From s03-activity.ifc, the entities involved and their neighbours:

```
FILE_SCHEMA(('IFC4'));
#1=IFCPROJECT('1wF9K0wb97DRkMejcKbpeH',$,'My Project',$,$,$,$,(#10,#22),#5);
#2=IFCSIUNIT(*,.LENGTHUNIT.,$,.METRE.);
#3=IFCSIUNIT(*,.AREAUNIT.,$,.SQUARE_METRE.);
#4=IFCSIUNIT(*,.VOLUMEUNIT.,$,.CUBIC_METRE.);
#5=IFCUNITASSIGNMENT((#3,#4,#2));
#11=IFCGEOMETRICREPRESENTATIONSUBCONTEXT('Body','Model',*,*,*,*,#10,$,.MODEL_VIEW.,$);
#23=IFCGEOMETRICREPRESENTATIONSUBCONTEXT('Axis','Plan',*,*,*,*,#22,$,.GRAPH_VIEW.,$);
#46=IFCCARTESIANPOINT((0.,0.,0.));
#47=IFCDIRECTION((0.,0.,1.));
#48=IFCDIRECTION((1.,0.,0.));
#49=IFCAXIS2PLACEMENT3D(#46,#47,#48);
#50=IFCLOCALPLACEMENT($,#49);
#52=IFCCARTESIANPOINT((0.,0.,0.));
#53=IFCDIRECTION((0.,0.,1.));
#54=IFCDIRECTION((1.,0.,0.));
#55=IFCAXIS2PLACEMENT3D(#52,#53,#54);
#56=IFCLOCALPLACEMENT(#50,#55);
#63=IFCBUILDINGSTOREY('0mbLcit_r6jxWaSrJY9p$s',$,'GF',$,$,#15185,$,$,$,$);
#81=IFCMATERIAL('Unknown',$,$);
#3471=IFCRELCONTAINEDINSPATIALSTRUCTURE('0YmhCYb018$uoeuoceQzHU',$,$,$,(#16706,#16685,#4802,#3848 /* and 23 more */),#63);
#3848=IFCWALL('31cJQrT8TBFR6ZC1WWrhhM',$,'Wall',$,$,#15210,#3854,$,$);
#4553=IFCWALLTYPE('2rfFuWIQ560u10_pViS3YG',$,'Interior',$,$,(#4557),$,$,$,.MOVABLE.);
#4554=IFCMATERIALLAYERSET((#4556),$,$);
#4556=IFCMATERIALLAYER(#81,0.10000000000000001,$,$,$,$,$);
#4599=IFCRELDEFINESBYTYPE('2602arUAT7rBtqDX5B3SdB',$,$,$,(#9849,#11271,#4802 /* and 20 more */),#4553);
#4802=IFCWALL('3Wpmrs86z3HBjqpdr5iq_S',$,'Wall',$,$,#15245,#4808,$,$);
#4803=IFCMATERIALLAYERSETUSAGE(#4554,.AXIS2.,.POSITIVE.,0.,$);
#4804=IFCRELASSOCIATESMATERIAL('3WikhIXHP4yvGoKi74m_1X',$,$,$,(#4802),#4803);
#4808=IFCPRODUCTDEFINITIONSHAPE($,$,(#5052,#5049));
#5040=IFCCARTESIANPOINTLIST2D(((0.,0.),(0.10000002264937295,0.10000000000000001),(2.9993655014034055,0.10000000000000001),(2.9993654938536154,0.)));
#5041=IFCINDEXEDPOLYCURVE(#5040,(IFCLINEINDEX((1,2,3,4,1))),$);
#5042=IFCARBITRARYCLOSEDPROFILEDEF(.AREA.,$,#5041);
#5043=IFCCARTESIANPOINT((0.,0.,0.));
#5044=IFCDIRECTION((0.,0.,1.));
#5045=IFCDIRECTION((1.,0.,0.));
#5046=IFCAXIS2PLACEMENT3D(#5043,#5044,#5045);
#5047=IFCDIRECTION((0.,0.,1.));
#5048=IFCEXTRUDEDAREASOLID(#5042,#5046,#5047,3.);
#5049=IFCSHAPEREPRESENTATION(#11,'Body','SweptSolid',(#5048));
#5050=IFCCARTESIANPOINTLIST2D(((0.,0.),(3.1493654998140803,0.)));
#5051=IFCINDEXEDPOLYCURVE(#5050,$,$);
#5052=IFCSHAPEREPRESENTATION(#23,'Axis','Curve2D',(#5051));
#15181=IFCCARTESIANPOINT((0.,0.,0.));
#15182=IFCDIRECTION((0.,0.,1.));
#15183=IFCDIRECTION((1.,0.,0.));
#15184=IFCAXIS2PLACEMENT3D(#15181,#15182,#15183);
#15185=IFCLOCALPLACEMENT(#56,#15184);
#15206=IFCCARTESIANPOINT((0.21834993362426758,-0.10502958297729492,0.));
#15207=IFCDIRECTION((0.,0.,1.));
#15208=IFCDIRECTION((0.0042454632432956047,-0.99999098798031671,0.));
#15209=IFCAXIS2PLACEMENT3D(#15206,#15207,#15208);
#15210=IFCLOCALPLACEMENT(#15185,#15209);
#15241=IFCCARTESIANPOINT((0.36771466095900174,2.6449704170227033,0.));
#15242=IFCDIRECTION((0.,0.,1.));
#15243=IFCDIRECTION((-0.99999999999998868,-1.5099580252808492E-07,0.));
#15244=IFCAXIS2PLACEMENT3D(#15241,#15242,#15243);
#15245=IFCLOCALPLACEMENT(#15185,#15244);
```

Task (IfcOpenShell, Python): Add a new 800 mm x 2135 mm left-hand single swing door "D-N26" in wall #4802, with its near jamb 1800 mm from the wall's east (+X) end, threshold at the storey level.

```python
import numpy as np
import ifcopenshell
import ifcopenshell.api.feature
import ifcopenshell.api.geometry
import ifcopenshell.api.root
import ifcopenshell.api.spatial
import ifcopenshell.geom
import ifcopenshell.util.element
import ifcopenshell.util.placement
import ifcopenshell.util.representation
import ifcopenshell.util.shape
import ifcopenshell.util.unit

model = ifcopenshell.open("s03-activity.ifc")
unit_scale = ifcopenshell.util.unit.calculate_unit_scale(model)
settings = ifcopenshell.geom.settings()


def volume(element):
    """Net volume in cubic metres, openings subtracted."""
    shape = ifcopenshell.geom.create_shape(settings, element)
    return ifcopenshell.util.shape.get_volume(shape.geometry)


wall = model.by_guid("3Wpmrs86z3HBjqpdr5iq_S")
storey = ifcopenshell.util.element.get_container(wall, ifc_class="IfcBuildingStorey")
context = ifcopenshell.util.representation.get_context(model, "Model", "Body", "MODEL_VIEW")
before = volume(wall)

width, height, from_end, sill = 0.8, 2.135, 1.8, 0.0  # metres

# The wall runs along its own X axis, and the end named is its -X end.
wall_shape = ifcopenshell.geom.create_shape(settings, wall)
x, y, z = ifcopenshell.util.shape.get_vertices(wall_shape.geometry).T
start = x.min() + from_end
face, thickness = float(y.min()), float(y.max() - y.min())
wall_matrix = ifcopenshell.util.placement.get_local_placement(wall.ObjectPlacement)
level = ifcopenshell.util.placement.get_local_placement(storey.ObjectPlacement)[2, 3]


def in_wall(x, y):
    """Placement at x, y metres in the wall's axes, at sill height."""
    matrix = wall_matrix.copy()
    matrix[:, 3] = wall_matrix @ np.array([x / unit_scale, y / unit_scale, 0.0, 1.0])
    matrix[2, 3] = level + sill / unit_scale
    return matrix


# Opening: a box that overshoots both wall faces by 50 mm.
opening = ifcopenshell.api.root.create_entity(model, ifc_class="IfcOpeningElement", predefined_type="OPENING")
box = ifcopenshell.api.geometry.add_wall_representation(
    model, context=context, length=width, height=height, thickness=thickness + 0.1
)
ifcopenshell.api.geometry.assign_representation(model, product=opening, representation=box)
ifcopenshell.api.geometry.edit_object_placement(model, product=opening, matrix=in_wall(start, face - 0.05), is_si=False)
ifcopenshell.api.feature.add_feature(model, feature=opening, element=wall)

door = ifcopenshell.api.root.create_entity(model, ifc_class="IfcDoor", name="D-N26", predefined_type="DOOR")
door.OverallWidth, door.OverallHeight = width / unit_scale, height / unit_scale
door.OperationType = "SINGLE_SWING_LEFT"
body = ifcopenshell.api.geometry.add_door_representation(
    model,
    context=context,
    overall_width=door.OverallWidth,
    overall_height=door.OverallHeight,
    operation_type="SINGLE_SWING_LEFT",
    lining_properties={"LiningDepth": thickness / unit_scale, "ThresholdDepth": thickness / unit_scale},
)
ifcopenshell.api.geometry.assign_representation(model, product=door, representation=body)
ifcopenshell.api.spatial.assign_container(model, products=[door], relating_structure=storey)
ifcopenshell.api.feature.add_filling(model, opening=opening, element=door)

# The lining spans the wall, so the door starts at the wall face.
ifcopenshell.api.geometry.edit_object_placement(model, product=door, matrix=in_wall(start, face), is_si=False)

after = volume(wall)

print(f"wall volume {before:.3f} -> {after:.3f} m3")

model.write("s03-activity_v2.ifc")
```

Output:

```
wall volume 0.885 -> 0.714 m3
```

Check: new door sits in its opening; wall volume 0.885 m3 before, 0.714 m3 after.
